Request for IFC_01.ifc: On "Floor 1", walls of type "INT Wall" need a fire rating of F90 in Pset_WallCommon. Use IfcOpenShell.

First a look at what the model holds.

```python
import ifcopenshell
import ifcopenshell.util.element

model = ifcopenshell.open("IFC_01.ifc")
print(model.schema)
storey = next(s for s in model.by_type("IfcBuildingStorey") if s.Name == "Floor 1")
walls = [e for e in ifcopenshell.util.element.get_decomposition(storey) if e.is_a("IfcWall")]
seen = {}
for e in walls:
    element_type = ifcopenshell.util.element.get_type(e)
    key = (element_type.Name if element_type != e and element_type else None, ifcopenshell.util.element.get_pset(e, "Pset_WallCommon", "FireRating"))
    seen[key] = seen.get(key, 0) + 1
for (name, value), count in sorted(seen.items(), key=str):
    print(count, "x", name, "|", value)
```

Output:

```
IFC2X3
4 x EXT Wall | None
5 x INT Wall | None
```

```python
import ifcopenshell
import ifcopenshell.api.pset
import ifcopenshell.util.element

model = ifcopenshell.open("IFC_01.ifc")

storey = next(s for s in model.by_type("IfcBuildingStorey") if s.Name == "Floor 1")
walls = [e for e in ifcopenshell.util.element.get_decomposition(storey) if e.is_a("IfcWall")]

count = 0
for e in walls:
    element_type = ifcopenshell.util.element.get_type(e)
    if element_type in (None, e) or element_type.Name != "INT Wall":
        continue
    # add_pset returns the element's existing set when there is one.
    pset = ifcopenshell.api.pset.add_pset(model, product=e, name="Pset_WallCommon")
    ifcopenshell.api.pset.edit_pset(model, pset=pset, properties={"FireRating": "F90"})
    count += 1

print(count, "walls updated")

model.write("IFC_01-out.ifc")
```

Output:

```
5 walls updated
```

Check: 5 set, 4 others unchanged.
